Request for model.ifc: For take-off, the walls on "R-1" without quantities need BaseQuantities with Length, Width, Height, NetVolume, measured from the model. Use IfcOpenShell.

First a look at what the model holds.

```python
import ifcopenshell
import ifcopenshell.util.element
import ifcopenshell.util.unit

model = ifcopenshell.open("model.ifc")
print(model.schema)
for unit_type in ("LENGTHUNIT", "AREAUNIT", "VOLUMEUNIT"):
    print(unit_type, ifcopenshell.util.unit.calculate_unit_scale(model, unit_type))
storey = next(s for s in model.by_type("IfcBuildingStorey") if s.Name == "R-1")
walls = [e for e in ifcopenshell.util.element.get_decomposition(storey) if e.is_a("IfcWall")]
for e in sorted(walls, key=lambda e: e.id()):
    print(e.id(), e.is_a(), e.Name, list(ifcopenshell.util.element.get_psets(e, qtos_only=True)), sep=" | ")
```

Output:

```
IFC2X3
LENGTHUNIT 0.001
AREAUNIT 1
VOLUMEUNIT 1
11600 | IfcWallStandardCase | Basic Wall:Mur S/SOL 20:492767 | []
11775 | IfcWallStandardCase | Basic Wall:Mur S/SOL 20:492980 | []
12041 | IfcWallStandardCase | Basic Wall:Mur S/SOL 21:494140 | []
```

```python
import ifcopenshell
import ifcopenshell.api.pset
import ifcopenshell.geom
import ifcopenshell.util.element
import ifcopenshell.util.shape
import ifcopenshell.util.unit

model = ifcopenshell.open("model.ifc")
unit_scale = ifcopenshell.util.unit.calculate_unit_scale(model)
volume_scale = ifcopenshell.util.unit.calculate_unit_scale(model, "VOLUMEUNIT")
settings = ifcopenshell.geom.settings()

storey = next(s for s in model.by_type("IfcBuildingStorey") if s.Name == "R-1")
walls = [e for e in ifcopenshell.util.element.get_decomposition(storey) if e.is_a("IfcWall")]

for e in sorted(walls, key=lambda e: e.id()):
    if ifcopenshell.util.element.get_psets(e, qtos_only=True, should_inherit=False):
        continue
    # Geometry comes back in metres, in the element's own axes.
    shape = ifcopenshell.geom.create_shape(settings, e)
    values = {
        "Length": ifcopenshell.util.shape.get_x(shape.geometry) / unit_scale,
        "Width": ifcopenshell.util.shape.get_y(shape.geometry) / unit_scale,
        "Height": ifcopenshell.util.shape.get_z(shape.geometry) / unit_scale,
        "NetVolume": ifcopenshell.util.shape.get_volume(shape.geometry) / volume_scale,
    }
    qto = ifcopenshell.api.pset.add_qto(model, product=e, name="BaseQuantities")
    ifcopenshell.api.pset.edit_qto(model, qto=qto, properties=values)
    print(e.id(), {k: round(v, 3) for k, v in values.items()})

model.write("model-out.ifc")
```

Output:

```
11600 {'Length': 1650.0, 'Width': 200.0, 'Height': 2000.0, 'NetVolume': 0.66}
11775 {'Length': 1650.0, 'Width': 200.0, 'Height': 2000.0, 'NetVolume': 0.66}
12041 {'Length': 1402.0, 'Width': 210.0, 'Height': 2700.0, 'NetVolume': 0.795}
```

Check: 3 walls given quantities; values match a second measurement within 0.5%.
